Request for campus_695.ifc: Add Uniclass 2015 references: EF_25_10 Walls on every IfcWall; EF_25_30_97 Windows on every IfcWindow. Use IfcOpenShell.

First a look at what the model holds.

```python
import ifcopenshell

model = ifcopenshell.open("campus_695.ifc")
print(model.schema)
print("classifications:", [c.Name for c in model.by_type("IfcClassification")])
for ifc_class in ("IfcDoor", "IfcRoof", "IfcStair", "IfcWall", "IfcWindow"):
    print(ifc_class, len(model.by_type(ifc_class)))
```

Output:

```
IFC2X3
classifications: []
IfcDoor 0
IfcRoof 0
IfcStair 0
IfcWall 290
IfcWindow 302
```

```python
import ifcopenshell
import ifcopenshell.api.classification

model = ifcopenshell.open("campus_695.ifc")

# IFC2X3 requires Source and Edition and has no link from the project to the system.
system = model.create_entity("IfcClassification", Source="NBS", Edition="2015", Name="Uniclass 2015")

codes = {
    "IfcWall": ("EF_25_10", "Walls"),
    "IfcWindow": ("EF_25_30_97", "Windows"),
}
for ifc_class, (code, name) in codes.items():
    products = model.by_type(ifc_class)
    ifcopenshell.api.classification.add_reference(
        model, products=products, classification=system, identification=code, name=name
    )
    print(code, len(products))

model.write("campus_695_rev.ifc")
```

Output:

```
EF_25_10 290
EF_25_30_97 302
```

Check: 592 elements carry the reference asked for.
